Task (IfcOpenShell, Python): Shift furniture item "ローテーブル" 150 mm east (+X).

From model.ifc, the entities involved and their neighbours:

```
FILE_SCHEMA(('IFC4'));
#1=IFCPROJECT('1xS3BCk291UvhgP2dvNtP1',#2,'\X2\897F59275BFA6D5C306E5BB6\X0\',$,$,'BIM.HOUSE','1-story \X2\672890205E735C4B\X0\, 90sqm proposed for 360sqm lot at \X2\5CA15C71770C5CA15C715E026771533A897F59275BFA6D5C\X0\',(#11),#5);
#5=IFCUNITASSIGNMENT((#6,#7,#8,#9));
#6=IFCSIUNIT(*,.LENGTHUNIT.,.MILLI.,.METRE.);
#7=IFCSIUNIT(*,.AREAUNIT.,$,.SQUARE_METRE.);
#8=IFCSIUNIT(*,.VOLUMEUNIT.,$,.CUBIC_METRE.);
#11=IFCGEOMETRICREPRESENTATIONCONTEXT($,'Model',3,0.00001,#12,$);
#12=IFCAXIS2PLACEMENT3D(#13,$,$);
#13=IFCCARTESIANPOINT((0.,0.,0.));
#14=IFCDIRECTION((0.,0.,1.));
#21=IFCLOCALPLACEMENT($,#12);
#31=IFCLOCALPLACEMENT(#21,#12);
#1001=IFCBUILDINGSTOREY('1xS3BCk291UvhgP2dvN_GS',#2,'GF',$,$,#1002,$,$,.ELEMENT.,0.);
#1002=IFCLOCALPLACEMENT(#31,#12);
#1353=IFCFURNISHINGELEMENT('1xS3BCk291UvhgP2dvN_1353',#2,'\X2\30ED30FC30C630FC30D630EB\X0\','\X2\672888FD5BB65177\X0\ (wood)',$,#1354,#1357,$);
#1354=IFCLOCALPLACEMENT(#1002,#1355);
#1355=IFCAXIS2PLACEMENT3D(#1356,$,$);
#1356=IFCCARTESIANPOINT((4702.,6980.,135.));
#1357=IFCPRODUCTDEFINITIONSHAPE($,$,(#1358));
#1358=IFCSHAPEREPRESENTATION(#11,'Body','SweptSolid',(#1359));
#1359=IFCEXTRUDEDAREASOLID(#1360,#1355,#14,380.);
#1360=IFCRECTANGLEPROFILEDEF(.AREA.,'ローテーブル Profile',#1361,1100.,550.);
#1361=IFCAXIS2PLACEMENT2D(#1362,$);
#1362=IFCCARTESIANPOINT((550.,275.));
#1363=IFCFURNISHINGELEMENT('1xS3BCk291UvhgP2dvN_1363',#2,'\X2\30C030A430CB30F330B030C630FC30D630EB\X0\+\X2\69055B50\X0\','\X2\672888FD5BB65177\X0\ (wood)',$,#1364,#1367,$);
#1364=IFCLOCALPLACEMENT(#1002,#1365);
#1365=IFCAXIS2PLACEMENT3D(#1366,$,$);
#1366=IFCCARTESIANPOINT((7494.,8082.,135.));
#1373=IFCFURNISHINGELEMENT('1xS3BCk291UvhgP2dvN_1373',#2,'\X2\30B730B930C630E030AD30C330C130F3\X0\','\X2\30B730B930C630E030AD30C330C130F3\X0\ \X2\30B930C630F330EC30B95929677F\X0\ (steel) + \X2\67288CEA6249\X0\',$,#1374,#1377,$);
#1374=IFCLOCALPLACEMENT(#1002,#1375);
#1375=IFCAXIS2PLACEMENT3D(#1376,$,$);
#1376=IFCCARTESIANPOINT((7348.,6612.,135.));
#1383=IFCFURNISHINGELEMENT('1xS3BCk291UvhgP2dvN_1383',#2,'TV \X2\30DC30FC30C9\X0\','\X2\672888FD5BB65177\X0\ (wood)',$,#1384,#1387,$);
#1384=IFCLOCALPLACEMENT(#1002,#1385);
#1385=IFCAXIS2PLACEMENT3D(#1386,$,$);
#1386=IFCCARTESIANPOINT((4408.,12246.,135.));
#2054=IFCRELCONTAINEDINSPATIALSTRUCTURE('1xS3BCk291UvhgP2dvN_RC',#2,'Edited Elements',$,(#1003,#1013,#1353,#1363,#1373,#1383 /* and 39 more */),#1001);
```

```python
import ifcopenshell
import ifcopenshell.api.geometry
import ifcopenshell.util.placement

model = ifcopenshell.open("model.ifc")

item = model.by_guid("1xS3BCk291UvhgP2dvN_1353")
matrix = ifcopenshell.util.placement.get_local_placement(item.ObjectPlacement)
matrix[0, 3] += 150.0
ifcopenshell.api.geometry.edit_object_placement(model, product=item, matrix=matrix, is_si=False)

print(ifcopenshell.util.placement.get_local_placement(item.ObjectPlacement).round(3) + 0.0)

model.write("model-out.ifc")
```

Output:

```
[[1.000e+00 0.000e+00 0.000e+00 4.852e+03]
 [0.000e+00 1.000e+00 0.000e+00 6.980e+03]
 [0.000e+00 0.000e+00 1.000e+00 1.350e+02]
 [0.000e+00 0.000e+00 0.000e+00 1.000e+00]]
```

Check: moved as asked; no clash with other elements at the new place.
